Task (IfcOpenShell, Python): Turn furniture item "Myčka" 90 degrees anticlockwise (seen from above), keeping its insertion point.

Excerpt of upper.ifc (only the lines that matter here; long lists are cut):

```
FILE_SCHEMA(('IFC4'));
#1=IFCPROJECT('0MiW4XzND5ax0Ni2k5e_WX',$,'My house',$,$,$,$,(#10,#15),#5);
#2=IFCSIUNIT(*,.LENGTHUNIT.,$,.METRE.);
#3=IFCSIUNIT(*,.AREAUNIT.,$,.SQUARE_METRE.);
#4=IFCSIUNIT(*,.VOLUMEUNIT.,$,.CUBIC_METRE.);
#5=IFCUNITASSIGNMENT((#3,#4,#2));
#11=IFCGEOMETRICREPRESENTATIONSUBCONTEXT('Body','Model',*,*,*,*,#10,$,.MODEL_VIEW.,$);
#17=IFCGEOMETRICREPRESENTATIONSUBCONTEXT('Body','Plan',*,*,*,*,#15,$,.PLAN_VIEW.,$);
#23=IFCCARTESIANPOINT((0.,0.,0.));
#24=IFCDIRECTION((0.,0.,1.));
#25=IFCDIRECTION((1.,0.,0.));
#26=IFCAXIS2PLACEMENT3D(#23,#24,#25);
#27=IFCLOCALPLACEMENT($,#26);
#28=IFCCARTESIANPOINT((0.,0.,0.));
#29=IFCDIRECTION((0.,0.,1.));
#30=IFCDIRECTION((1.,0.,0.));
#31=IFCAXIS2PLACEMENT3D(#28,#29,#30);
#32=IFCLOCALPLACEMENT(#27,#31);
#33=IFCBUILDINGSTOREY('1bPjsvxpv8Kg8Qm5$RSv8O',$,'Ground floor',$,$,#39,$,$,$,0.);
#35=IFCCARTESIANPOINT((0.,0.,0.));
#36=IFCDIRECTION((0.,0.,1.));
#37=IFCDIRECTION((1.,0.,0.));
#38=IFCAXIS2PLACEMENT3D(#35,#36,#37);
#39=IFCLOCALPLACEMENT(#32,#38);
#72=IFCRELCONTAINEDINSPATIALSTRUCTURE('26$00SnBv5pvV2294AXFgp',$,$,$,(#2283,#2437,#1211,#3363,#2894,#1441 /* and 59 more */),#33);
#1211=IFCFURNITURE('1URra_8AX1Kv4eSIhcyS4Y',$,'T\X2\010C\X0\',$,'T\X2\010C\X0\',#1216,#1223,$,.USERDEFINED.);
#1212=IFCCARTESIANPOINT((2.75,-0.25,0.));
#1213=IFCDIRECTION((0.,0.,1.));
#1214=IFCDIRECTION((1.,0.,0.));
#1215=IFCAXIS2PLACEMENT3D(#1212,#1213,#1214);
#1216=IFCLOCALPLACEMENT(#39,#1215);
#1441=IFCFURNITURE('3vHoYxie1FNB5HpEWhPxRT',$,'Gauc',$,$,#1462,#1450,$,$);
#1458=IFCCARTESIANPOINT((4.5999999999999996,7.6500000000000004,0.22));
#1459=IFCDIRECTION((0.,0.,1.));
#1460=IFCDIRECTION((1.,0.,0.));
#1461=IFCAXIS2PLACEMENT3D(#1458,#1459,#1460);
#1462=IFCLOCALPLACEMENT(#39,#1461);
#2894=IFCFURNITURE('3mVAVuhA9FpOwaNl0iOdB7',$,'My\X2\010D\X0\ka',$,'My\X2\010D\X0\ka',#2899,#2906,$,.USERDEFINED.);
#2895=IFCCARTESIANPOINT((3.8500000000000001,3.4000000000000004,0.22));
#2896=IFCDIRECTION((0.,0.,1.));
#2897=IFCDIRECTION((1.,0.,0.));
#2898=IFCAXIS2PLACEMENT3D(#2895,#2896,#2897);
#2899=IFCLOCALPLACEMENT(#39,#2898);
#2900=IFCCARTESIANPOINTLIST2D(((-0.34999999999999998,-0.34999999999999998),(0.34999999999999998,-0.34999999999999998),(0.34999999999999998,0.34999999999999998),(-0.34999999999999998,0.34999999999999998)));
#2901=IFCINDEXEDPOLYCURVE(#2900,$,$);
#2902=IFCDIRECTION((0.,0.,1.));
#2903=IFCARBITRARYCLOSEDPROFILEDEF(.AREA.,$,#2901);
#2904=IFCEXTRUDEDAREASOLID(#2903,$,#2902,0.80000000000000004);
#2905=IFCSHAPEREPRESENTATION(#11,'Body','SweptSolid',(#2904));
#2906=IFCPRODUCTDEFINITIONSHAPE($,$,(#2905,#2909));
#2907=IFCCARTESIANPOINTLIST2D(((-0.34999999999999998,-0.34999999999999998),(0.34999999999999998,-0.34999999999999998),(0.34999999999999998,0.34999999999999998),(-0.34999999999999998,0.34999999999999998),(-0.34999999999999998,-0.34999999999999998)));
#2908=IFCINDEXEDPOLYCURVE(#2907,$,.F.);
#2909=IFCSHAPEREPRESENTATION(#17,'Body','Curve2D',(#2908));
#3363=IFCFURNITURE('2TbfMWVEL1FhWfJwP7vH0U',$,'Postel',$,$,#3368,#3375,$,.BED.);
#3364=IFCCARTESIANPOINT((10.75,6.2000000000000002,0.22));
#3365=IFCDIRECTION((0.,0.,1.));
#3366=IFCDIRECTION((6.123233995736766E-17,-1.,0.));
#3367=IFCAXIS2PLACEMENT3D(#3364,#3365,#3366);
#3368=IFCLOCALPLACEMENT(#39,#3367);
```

```python
import ifcopenshell
import ifcopenshell.api.geometry
import ifcopenshell.util.placement

model = ifcopenshell.open("upper.ifc")

item = model.by_id(2894)
matrix = ifcopenshell.util.placement.get_local_placement(item.ObjectPlacement)
matrix = matrix @ ifcopenshell.util.placement.rotation(90, "Z")
ifcopenshell.api.geometry.edit_object_placement(model, product=item, matrix=matrix, is_si=False)

print(ifcopenshell.util.placement.get_local_placement(item.ObjectPlacement).round(3) + 0.0)

model.write("upper_updated.ifc")
```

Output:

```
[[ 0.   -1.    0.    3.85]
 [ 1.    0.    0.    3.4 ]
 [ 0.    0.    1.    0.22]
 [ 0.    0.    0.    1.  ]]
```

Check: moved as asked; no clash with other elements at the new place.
